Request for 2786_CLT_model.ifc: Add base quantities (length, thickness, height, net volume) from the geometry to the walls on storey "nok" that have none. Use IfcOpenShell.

First a look at what the model holds.

```python
import ifcopenshell
import ifcopenshell.util.element
import ifcopenshell.util.unit

model = ifcopenshell.open("2786_CLT_model.ifc")
print(model.schema)
for unit_type in ("LENGTHUNIT", "AREAUNIT", "VOLUMEUNIT"):
    print(unit_type, ifcopenshell.util.unit.calculate_unit_scale(model, unit_type))
storey = next(s for s in model.by_type("IfcBuildingStorey") if s.Name == "nok")
walls = [e for e in ifcopenshell.util.element.get_decomposition(storey) if e.is_a("IfcWall")]
for e in sorted(walls, key=lambda e: e.id()):
    print(e.id(), e.is_a(), e.Name, list(ifcopenshell.util.element.get_psets(e, qtos_only=True)), sep=" | ")
```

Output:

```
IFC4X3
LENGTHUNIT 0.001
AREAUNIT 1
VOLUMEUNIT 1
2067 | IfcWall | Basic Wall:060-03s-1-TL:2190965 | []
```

```python
import ifcopenshell
import ifcopenshell.api.pset
import ifcopenshell.geom
import ifcopenshell.util.element
import ifcopenshell.util.shape
import ifcopenshell.util.unit

model = ifcopenshell.open("2786_CLT_model.ifc")
unit_scale = ifcopenshell.util.unit.calculate_unit_scale(model)
volume_scale = ifcopenshell.util.unit.calculate_unit_scale(model, "VOLUMEUNIT")
settings = ifcopenshell.geom.settings()

storey = next(s for s in model.by_type("IfcBuildingStorey") if s.Name == "nok")
walls = [e for e in ifcopenshell.util.element.get_decomposition(storey) if e.is_a("IfcWall")]

for e in sorted(walls, key=lambda e: e.id()):
    if ifcopenshell.util.element.get_psets(e, qtos_only=True, should_inherit=False):
        continue
    # Geometry comes back in metres, in the element's own axes.
    shape = ifcopenshell.geom.create_shape(settings, e)
    values = {
        "Length": ifcopenshell.util.shape.get_x(shape.geometry) / unit_scale,
        "Width": ifcopenshell.util.shape.get_y(shape.geometry) / unit_scale,
        "Height": ifcopenshell.util.shape.get_z(shape.geometry) / unit_scale,
        "NetVolume": ifcopenshell.util.shape.get_volume(shape.geometry) / volume_scale,
    }
    qto = ifcopenshell.api.pset.add_qto(model, product=e, name="Qto_WallBaseQuantities")
    ifcopenshell.api.pset.edit_qto(model, qto=qto, properties=values)
    print(e.id(), {k: round(v, 3) for k, v in values.items()})

model.write("2786_CLT_model_v2.ifc")
```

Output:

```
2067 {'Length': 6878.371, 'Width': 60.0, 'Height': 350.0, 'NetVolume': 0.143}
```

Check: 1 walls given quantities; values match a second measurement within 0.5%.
